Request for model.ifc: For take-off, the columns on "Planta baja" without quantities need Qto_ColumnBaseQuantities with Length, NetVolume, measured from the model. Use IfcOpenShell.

First a look at what the model holds.

```python
import ifcopenshell
import ifcopenshell.util.element
import ifcopenshell.util.unit

model = ifcopenshell.open("model.ifc")
print(model.schema)
for unit_type in ("LENGTHUNIT", "AREAUNIT", "VOLUMEUNIT"):
    print(unit_type, ifcopenshell.util.unit.calculate_unit_scale(model, unit_type))
storey = next(s for s in model.by_type("IfcBuildingStorey") if s.Name == "Planta baja")
columns = [e for e in ifcopenshell.util.element.get_decomposition(storey) if e.is_a("IfcColumn")]
for e in sorted(columns, key=lambda e: e.id()):
    print(e.id(), e.is_a(), e.Name, list(ifcopenshell.util.element.get_psets(e, qtos_only=True)), sep=" | ")
```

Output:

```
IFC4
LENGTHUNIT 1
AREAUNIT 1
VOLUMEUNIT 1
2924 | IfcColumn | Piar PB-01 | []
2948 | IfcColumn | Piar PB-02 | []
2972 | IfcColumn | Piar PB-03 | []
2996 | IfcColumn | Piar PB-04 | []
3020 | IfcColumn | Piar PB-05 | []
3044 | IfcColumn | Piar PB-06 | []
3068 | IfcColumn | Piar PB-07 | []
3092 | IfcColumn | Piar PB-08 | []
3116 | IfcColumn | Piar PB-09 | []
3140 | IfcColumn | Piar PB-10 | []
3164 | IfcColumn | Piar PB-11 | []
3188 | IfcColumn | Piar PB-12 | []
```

```python
import ifcopenshell
import ifcopenshell.api.pset
import ifcopenshell.geom
import ifcopenshell.util.element
import ifcopenshell.util.shape
import ifcopenshell.util.unit

model = ifcopenshell.open("model.ifc")
unit_scale = ifcopenshell.util.unit.calculate_unit_scale(model)
volume_scale = ifcopenshell.util.unit.calculate_unit_scale(model, "VOLUMEUNIT")
settings = ifcopenshell.geom.settings()

storey = next(s for s in model.by_type("IfcBuildingStorey") if s.Name == "Planta baja")
columns = [e for e in ifcopenshell.util.element.get_decomposition(storey) if e.is_a("IfcColumn")]

for e in sorted(columns, key=lambda e: e.id()):
    if ifcopenshell.util.element.get_psets(e, qtos_only=True, should_inherit=False):
        continue
    # Geometry comes back in metres, in the element's own axes.
    shape = ifcopenshell.geom.create_shape(settings, e)
    values = {
        "Length": ifcopenshell.util.shape.get_z(shape.geometry) / unit_scale,
        "NetVolume": ifcopenshell.util.shape.get_volume(shape.geometry) / volume_scale,
    }
    qto = ifcopenshell.api.pset.add_qto(model, product=e, name="Qto_ColumnBaseQuantities")
    ifcopenshell.api.pset.edit_qto(model, qto=qto, properties=values)
    print(e.id(), {k: round(v, 3) for k, v in values.items()})

model.write("model-out.ifc")
```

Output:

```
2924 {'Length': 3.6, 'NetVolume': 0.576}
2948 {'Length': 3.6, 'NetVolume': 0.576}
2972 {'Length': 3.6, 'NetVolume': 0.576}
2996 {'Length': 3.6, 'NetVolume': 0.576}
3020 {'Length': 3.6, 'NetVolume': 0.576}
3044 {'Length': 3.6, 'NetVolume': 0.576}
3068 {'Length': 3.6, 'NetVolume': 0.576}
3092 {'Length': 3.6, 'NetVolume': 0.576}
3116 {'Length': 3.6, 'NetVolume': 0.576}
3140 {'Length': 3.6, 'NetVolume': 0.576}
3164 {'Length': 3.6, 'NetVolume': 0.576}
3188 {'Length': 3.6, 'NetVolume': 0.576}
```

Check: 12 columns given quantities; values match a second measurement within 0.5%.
